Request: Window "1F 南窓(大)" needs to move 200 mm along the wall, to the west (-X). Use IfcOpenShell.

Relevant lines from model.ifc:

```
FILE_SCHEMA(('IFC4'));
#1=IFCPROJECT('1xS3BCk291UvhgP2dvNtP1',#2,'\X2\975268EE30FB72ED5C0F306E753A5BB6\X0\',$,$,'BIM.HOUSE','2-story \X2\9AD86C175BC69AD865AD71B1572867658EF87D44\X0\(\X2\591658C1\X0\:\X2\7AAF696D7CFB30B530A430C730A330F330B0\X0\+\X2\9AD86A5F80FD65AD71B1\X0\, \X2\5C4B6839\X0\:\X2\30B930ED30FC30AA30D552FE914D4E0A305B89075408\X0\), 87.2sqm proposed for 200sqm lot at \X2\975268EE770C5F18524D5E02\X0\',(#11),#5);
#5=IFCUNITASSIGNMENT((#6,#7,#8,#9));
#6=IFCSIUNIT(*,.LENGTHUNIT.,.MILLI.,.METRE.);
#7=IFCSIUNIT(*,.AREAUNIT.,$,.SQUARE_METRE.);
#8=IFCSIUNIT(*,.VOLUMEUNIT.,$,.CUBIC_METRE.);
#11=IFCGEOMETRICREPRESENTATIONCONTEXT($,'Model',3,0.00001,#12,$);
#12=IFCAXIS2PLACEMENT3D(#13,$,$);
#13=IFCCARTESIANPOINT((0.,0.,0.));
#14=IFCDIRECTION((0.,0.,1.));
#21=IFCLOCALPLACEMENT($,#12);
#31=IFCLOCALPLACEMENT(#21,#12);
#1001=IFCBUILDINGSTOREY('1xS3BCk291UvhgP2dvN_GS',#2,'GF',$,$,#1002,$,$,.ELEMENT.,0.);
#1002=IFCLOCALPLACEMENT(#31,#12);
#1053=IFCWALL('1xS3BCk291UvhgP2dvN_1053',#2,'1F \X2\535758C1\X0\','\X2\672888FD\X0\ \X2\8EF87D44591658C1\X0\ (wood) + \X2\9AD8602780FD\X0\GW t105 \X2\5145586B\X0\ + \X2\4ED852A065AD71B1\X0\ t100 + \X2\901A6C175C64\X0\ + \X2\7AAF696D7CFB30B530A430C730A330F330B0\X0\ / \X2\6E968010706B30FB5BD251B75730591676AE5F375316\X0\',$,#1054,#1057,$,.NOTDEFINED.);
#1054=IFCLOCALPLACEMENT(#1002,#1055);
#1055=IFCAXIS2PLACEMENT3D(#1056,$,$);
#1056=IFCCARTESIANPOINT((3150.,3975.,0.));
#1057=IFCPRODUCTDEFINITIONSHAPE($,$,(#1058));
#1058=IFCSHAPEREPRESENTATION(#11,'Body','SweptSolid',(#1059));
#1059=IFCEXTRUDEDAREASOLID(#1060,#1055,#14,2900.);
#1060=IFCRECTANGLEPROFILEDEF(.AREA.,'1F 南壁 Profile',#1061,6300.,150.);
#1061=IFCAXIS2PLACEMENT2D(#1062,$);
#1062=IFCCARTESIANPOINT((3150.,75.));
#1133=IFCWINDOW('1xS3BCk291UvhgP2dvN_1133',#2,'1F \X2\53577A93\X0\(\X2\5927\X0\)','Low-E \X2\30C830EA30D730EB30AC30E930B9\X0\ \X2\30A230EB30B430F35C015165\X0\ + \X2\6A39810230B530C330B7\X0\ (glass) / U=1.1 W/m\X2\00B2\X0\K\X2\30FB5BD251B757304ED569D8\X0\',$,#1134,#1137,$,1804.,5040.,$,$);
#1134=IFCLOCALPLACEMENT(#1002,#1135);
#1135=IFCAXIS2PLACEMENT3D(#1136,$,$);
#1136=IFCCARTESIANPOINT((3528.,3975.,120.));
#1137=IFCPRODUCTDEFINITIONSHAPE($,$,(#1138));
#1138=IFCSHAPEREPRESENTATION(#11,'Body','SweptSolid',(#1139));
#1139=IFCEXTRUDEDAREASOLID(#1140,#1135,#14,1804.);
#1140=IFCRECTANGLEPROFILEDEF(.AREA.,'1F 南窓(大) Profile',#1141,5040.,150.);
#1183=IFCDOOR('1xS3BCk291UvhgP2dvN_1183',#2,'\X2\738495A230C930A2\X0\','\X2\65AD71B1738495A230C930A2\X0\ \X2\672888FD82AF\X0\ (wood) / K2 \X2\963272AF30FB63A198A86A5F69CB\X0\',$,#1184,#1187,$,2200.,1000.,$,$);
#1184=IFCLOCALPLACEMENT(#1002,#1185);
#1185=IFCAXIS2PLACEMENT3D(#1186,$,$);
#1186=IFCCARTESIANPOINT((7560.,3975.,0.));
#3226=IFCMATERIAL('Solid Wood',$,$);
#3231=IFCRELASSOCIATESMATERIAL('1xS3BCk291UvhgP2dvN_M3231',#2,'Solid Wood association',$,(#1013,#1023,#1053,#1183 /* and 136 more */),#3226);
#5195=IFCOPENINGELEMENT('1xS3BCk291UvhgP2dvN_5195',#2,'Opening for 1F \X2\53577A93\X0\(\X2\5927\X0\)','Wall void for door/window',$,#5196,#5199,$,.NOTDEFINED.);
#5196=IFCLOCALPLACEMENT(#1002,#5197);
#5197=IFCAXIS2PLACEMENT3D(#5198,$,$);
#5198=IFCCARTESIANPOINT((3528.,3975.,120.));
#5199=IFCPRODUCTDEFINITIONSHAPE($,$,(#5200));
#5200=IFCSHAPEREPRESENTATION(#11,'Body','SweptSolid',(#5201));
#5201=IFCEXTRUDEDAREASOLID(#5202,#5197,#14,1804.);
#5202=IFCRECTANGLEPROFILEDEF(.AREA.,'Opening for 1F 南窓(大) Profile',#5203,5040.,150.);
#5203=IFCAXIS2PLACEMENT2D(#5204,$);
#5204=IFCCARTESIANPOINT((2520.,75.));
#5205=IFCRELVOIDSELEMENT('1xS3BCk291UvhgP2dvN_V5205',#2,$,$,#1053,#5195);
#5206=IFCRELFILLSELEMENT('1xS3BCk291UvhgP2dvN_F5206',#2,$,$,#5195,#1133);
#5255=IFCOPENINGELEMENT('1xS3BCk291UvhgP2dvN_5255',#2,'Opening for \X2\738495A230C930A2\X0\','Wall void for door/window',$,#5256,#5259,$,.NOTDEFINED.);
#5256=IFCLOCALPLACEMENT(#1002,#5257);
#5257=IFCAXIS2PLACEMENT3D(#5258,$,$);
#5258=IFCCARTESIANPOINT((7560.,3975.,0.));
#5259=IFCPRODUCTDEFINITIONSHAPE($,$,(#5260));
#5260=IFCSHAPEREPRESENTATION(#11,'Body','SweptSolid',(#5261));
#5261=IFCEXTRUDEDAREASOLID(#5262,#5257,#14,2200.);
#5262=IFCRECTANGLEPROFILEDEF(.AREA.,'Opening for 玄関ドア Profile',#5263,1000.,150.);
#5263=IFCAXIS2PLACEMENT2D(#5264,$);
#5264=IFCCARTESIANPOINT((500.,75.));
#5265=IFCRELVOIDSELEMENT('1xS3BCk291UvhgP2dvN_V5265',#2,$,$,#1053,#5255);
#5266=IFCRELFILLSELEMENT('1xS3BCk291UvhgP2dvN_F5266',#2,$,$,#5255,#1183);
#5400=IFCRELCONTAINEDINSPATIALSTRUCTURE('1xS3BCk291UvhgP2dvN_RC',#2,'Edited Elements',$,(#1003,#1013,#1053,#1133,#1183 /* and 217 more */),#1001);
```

```python
import ifcopenshell
import ifcopenshell.api.geometry
import ifcopenshell.util.placement
import ifcopenshell.util.unit

model = ifcopenshell.open("model.ifc")
unit_scale = ifcopenshell.util.unit.calculate_unit_scale(model)

window = model.by_id(1133)
opening = window.FillsVoids[0].RelatingOpeningElement
wall = opening.VoidsElements[0].RelatingBuildingElement

wall_matrix = ifcopenshell.util.placement.get_local_placement(wall.ObjectPlacement)
shift = wall_matrix[:3, 0] * -0.2 / unit_scale
before = ifcopenshell.util.placement.get_local_placement(window.ObjectPlacement)[:3, 3].copy()

# The window is not placed relative to its opening, so move both.
for product in (opening, window):
    matrix = ifcopenshell.util.placement.get_local_placement(product.ObjectPlacement)
    matrix[:3, 3] += shift
    ifcopenshell.api.geometry.edit_object_placement(model, product=product, matrix=matrix, is_si=False)

after = ifcopenshell.util.placement.get_local_placement(window.ObjectPlacement)[:3, 3]
print("window moved by", (after - before).round(3) + 0.0)

model.write("model-out.ifc")
```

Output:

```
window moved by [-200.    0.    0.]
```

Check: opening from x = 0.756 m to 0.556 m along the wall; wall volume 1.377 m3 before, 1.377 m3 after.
